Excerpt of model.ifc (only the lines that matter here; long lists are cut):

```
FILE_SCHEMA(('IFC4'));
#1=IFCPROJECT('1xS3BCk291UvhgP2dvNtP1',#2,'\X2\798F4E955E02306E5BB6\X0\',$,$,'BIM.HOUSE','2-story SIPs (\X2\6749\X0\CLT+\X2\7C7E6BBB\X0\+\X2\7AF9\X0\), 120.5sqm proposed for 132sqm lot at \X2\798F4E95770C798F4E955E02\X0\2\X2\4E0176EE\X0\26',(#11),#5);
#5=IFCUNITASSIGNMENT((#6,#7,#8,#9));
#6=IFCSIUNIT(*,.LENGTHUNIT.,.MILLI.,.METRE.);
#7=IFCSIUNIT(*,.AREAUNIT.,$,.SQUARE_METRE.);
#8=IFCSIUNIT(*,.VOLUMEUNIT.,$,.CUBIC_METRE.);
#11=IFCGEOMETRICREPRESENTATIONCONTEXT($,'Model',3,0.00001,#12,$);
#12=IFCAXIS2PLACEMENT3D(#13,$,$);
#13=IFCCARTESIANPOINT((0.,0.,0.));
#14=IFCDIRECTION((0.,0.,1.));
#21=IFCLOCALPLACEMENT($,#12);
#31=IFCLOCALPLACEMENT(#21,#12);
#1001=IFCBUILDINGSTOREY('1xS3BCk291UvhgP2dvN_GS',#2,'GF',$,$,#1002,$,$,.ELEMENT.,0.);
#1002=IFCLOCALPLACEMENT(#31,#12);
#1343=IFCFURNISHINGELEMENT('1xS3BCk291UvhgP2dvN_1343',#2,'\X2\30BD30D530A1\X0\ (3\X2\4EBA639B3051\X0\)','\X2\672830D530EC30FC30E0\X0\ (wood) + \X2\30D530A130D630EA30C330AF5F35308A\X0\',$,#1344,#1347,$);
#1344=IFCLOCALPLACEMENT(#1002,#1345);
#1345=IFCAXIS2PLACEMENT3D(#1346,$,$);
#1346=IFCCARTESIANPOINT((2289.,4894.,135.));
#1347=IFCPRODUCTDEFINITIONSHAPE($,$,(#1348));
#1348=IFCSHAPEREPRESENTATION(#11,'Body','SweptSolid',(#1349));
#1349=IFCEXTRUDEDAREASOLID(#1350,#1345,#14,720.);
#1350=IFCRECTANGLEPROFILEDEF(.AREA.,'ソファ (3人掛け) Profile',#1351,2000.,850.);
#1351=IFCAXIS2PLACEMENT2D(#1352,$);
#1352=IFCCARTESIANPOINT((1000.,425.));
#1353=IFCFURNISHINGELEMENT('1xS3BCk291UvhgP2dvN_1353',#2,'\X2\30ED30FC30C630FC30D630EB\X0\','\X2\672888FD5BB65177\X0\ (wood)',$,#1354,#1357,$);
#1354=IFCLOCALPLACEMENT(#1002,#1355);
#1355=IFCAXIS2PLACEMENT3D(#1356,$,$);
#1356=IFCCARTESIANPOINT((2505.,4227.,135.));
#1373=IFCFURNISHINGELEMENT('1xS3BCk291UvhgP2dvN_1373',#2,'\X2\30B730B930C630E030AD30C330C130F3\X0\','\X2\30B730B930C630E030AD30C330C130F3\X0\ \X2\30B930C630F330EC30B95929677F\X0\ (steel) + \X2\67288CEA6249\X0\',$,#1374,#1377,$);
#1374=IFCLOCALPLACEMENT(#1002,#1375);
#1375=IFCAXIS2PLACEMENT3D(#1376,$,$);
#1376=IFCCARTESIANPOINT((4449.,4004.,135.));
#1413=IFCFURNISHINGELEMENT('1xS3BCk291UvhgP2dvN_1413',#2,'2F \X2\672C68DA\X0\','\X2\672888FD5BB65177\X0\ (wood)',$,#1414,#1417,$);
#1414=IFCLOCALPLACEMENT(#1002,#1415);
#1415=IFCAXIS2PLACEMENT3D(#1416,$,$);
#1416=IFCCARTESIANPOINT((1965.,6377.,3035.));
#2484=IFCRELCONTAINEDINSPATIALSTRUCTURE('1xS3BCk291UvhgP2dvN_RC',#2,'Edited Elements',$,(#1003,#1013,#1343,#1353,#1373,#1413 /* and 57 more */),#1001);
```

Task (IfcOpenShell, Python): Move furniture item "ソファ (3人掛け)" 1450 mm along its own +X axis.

```python
import ifcopenshell
import ifcopenshell.api.geometry
import ifcopenshell.util.placement

model = ifcopenshell.open("model.ifc")

item = model.by_id(1343)
matrix = ifcopenshell.util.placement.get_local_placement(item.ObjectPlacement)
matrix[:3, 3] += matrix[:3, 0] * 1450.0
ifcopenshell.api.geometry.edit_object_placement(model, product=item, matrix=matrix, is_si=False)

print(ifcopenshell.util.placement.get_local_placement(item.ObjectPlacement).round(3) + 0.0)

model.write("model_v2.ifc")
```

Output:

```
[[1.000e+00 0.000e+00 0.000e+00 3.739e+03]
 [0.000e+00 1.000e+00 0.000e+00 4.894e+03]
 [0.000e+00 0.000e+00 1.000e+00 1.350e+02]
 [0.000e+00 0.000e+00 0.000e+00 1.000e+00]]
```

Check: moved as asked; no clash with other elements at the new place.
